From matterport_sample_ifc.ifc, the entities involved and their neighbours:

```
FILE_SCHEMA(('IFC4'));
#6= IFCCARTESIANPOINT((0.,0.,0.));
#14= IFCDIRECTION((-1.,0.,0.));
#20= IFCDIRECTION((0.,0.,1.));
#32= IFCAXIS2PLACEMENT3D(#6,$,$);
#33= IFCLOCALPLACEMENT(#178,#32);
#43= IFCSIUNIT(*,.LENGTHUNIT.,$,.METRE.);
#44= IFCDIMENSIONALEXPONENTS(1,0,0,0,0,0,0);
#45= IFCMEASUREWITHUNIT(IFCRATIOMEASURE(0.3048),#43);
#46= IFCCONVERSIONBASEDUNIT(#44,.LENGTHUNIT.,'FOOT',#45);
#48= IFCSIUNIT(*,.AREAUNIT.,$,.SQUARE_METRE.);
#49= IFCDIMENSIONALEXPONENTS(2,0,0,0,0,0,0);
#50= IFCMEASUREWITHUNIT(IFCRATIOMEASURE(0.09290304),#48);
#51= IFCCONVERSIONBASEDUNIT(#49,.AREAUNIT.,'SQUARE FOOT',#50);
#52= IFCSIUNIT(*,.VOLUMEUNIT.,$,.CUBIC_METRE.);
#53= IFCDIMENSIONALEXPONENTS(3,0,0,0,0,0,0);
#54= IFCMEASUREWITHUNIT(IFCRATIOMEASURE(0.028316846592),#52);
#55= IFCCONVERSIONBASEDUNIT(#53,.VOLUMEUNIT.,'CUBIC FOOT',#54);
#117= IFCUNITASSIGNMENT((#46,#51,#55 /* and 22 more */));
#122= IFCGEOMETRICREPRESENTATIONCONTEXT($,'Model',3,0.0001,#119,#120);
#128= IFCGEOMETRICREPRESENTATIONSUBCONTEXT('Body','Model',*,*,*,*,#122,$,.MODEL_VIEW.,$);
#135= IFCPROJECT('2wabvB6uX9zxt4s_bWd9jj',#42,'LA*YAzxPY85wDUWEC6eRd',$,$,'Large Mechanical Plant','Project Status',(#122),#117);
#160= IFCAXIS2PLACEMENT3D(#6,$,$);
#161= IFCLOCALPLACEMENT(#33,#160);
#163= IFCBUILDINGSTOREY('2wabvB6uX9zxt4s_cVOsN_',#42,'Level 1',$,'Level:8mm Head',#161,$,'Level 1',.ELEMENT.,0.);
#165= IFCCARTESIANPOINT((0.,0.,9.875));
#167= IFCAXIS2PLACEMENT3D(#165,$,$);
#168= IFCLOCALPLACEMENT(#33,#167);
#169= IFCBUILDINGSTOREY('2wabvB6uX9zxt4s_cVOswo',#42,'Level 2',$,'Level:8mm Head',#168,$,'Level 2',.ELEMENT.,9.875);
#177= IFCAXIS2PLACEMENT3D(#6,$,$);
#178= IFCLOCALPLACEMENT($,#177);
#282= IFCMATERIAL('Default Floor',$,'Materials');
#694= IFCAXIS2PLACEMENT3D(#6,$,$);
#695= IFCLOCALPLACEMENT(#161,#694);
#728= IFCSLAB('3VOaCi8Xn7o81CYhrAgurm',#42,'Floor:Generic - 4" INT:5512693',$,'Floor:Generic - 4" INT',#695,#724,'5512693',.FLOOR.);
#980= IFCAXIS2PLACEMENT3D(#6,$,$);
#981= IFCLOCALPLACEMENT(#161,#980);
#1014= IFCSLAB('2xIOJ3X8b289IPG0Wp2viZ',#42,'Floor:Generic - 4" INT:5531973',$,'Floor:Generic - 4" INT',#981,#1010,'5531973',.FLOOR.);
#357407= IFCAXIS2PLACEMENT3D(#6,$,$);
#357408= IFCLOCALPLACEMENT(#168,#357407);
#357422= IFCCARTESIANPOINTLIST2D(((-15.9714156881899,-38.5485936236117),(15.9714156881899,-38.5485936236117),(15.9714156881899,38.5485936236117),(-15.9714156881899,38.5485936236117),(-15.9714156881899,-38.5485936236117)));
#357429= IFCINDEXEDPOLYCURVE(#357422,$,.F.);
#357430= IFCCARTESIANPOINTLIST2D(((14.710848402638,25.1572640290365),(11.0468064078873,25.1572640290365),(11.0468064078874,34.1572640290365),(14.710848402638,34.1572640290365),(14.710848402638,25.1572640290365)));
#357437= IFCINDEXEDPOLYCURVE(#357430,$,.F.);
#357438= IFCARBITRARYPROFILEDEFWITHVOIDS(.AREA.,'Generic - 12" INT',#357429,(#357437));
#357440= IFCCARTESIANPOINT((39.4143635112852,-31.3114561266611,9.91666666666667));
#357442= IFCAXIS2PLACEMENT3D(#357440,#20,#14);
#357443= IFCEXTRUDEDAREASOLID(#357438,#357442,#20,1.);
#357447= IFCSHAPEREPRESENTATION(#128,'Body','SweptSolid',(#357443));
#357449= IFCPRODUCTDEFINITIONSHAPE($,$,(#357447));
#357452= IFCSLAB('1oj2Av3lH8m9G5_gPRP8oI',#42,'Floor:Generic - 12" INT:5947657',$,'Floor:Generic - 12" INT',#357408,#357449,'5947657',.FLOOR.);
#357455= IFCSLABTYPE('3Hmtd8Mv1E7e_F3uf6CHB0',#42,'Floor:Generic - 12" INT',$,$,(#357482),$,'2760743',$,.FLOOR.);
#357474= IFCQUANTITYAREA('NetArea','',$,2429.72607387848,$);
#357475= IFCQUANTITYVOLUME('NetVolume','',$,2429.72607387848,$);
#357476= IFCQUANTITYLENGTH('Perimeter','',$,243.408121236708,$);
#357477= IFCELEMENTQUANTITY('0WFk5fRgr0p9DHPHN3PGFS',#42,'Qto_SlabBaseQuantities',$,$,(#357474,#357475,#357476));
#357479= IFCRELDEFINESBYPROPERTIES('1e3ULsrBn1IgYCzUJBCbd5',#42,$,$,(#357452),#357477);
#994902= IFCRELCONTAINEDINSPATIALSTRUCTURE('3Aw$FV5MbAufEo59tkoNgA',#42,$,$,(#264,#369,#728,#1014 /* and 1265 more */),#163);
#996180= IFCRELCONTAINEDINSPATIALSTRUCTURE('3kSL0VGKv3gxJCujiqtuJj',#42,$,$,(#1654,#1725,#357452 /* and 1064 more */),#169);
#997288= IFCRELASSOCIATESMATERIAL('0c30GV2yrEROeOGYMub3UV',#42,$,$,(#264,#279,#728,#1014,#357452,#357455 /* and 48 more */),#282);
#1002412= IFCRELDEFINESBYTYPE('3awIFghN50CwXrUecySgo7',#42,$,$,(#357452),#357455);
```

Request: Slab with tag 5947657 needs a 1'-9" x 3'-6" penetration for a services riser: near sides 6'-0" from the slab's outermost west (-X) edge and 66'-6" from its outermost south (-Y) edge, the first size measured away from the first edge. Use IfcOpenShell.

```python
import numpy as np
import ifcopenshell
import ifcopenshell.api.feature
import ifcopenshell.api.geometry
import ifcopenshell.api.pset
import ifcopenshell.api.root
import ifcopenshell.geom
import ifcopenshell.util.element
import ifcopenshell.util.placement
import ifcopenshell.util.representation
import ifcopenshell.util.shape
import ifcopenshell.util.unit

model = ifcopenshell.open("matterport_sample_ifc.ifc")
unit_scale = ifcopenshell.util.unit.calculate_unit_scale(model)
area_scale = ifcopenshell.util.unit.calculate_unit_scale(model, "AREAUNIT")
volume_scale = ifcopenshell.util.unit.calculate_unit_scale(model, "VOLUMEUNIT")
settings = ifcopenshell.geom.settings()


def volume(element):
    """Net volume in cubic metres, openings subtracted."""
    shape = ifcopenshell.geom.create_shape(settings, element)
    return ifcopenshell.util.shape.get_volume(shape.geometry)


slab = model.by_guid("1oj2Av3lH8m9G5_gPRP8oI")
before = volume(slab)

# Extent in the slab's own axes, in metres. The edges named are its -X and -Y sides.
slab_shape = ifcopenshell.geom.create_shape(settings, slab)
vertices = ifcopenshell.util.shape.get_vertices(slab_shape.geometry)
x_min, y_min, bottom = vertices.min(axis=0)
top = vertices[:, 2].max()

opening = ifcopenshell.api.root.create_entity(model, ifc_class="IfcOpeningElement", name="Services riser opening", predefined_type="OPENING")
context = ifcopenshell.util.representation.get_context(model, "Model", "Body", "MODEL_VIEW")
width, depth = 0.5334, 1.0668
outline = [(0.0, 0.0), (width, 0.0), (width, depth), (0.0, depth), (0.0, 0.0)]
# Overshoot both faces by 50 mm so the cut is clean.
shape = ifcopenshell.api.geometry.add_slab_representation(
    model, context=context, depth=top - bottom + 0.1, polyline=outline
)
ifcopenshell.api.geometry.assign_representation(model, product=opening, representation=shape)

matrix = ifcopenshell.util.placement.get_local_placement(slab.ObjectPlacement)
matrix[:, 3] = matrix @ np.append(np.array([x_min + 1.8288, y_min + 20.2692, bottom - 0.05]) / unit_scale, 1.0)
ifcopenshell.api.geometry.edit_object_placement(model, product=opening, matrix=matrix, is_si=False)
ifcopenshell.api.feature.add_feature(model, feature=opening, element=slab)

after = volume(slab)

# Update the slab's stored quantities.
qto = model.by_id(ifcopenshell.util.element.get_pset(slab, "Qto_SlabBaseQuantities", should_inherit=False)["id"])
ifcopenshell.api.pset.edit_qto(model, qto=qto, properties={
    "NetArea": after / (top - bottom) / area_scale,
    "NetVolume": after / volume_scale,
})

print(f"slab volume {before:.3f} -> {after:.3f} m3")

model.write("matterport_sample_ifc_updated.ifc")
```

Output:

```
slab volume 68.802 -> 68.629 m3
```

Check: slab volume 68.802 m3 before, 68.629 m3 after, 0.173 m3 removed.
